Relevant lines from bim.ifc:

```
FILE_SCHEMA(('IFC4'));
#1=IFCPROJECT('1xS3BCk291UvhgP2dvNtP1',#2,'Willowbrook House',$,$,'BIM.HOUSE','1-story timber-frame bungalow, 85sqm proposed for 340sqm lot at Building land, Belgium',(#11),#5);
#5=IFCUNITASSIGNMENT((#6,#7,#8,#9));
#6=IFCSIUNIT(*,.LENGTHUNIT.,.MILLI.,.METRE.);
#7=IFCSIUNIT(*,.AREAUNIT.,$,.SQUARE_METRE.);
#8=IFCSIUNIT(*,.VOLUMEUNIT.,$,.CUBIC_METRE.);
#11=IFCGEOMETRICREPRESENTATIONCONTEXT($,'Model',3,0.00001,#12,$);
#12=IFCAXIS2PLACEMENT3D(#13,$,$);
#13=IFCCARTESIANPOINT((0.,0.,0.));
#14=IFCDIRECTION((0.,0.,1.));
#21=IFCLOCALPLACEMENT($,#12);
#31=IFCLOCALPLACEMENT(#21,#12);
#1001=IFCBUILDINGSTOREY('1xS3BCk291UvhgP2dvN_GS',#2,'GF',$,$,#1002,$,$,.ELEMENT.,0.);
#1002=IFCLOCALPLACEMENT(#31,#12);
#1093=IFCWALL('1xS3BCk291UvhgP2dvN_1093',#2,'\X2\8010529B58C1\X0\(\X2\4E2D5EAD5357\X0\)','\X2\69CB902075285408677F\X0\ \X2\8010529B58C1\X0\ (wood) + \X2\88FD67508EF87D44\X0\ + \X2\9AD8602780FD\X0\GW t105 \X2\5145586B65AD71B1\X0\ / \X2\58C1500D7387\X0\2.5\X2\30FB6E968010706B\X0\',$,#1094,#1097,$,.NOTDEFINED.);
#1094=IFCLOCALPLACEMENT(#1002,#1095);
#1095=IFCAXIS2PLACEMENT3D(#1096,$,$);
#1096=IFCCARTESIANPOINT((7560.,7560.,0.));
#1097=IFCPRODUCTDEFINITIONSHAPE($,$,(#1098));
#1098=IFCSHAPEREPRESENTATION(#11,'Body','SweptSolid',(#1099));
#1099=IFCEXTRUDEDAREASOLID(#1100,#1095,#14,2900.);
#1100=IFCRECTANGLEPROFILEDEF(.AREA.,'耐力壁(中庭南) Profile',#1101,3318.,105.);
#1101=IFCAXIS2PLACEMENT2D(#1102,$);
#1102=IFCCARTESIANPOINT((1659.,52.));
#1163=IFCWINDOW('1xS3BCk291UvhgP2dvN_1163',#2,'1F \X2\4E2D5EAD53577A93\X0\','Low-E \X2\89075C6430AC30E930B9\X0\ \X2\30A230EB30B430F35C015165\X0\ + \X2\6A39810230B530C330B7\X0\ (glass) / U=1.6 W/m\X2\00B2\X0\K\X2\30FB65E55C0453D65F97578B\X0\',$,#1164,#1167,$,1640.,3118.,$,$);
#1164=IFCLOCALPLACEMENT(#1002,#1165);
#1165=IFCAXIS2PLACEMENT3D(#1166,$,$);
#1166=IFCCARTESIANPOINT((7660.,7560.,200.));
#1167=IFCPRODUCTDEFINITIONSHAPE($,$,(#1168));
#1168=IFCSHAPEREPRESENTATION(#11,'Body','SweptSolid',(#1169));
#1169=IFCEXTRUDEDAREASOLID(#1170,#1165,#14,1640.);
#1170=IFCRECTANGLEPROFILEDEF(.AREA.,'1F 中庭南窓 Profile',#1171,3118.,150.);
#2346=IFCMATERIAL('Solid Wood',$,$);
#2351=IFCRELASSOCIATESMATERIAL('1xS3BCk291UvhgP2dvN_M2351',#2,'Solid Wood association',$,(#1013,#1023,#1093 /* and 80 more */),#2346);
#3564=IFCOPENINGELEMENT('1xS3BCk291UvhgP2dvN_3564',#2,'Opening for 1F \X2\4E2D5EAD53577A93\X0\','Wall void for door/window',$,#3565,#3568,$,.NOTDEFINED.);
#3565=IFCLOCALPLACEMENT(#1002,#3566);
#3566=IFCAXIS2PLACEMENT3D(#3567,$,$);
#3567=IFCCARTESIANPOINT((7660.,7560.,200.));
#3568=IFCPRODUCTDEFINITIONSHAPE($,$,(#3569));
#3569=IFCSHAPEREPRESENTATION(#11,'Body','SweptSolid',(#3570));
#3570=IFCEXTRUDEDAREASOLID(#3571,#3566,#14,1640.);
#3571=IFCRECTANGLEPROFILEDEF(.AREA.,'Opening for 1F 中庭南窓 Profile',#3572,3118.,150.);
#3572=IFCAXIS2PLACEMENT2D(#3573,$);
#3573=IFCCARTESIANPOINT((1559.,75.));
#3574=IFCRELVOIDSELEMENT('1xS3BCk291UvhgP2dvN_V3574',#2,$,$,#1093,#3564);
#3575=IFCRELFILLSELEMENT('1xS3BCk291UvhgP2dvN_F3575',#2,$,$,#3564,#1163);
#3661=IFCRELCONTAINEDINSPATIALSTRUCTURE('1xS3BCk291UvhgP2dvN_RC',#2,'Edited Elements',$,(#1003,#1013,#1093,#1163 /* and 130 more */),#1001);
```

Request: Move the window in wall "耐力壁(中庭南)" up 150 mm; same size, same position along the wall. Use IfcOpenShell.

```python
import numpy as np
import ifcopenshell
import ifcopenshell.api.geometry
import ifcopenshell.util.placement
import ifcopenshell.util.unit

model = ifcopenshell.open("bim.ifc")
unit_scale = ifcopenshell.util.unit.calculate_unit_scale(model)

window = model.by_guid("1xS3BCk291UvhgP2dvN_1163")
opening = window.FillsVoids[0].RelatingOpeningElement
dz = 150.0

shift = np.array([0.0, 0.0, dz])
# The window is not placed relative to its opening, so move both.
for product in (opening, window):
    matrix = ifcopenshell.util.placement.get_local_placement(product.ObjectPlacement)
    matrix[:3, 3] += shift
    ifcopenshell.api.geometry.edit_object_placement(model, product=product, matrix=matrix, is_si=False)

print(f"moved by {dz * unit_scale:+.3f} m")

model.write("bim_v2.ifc")
```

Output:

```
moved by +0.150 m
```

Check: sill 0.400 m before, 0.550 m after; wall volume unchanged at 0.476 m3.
